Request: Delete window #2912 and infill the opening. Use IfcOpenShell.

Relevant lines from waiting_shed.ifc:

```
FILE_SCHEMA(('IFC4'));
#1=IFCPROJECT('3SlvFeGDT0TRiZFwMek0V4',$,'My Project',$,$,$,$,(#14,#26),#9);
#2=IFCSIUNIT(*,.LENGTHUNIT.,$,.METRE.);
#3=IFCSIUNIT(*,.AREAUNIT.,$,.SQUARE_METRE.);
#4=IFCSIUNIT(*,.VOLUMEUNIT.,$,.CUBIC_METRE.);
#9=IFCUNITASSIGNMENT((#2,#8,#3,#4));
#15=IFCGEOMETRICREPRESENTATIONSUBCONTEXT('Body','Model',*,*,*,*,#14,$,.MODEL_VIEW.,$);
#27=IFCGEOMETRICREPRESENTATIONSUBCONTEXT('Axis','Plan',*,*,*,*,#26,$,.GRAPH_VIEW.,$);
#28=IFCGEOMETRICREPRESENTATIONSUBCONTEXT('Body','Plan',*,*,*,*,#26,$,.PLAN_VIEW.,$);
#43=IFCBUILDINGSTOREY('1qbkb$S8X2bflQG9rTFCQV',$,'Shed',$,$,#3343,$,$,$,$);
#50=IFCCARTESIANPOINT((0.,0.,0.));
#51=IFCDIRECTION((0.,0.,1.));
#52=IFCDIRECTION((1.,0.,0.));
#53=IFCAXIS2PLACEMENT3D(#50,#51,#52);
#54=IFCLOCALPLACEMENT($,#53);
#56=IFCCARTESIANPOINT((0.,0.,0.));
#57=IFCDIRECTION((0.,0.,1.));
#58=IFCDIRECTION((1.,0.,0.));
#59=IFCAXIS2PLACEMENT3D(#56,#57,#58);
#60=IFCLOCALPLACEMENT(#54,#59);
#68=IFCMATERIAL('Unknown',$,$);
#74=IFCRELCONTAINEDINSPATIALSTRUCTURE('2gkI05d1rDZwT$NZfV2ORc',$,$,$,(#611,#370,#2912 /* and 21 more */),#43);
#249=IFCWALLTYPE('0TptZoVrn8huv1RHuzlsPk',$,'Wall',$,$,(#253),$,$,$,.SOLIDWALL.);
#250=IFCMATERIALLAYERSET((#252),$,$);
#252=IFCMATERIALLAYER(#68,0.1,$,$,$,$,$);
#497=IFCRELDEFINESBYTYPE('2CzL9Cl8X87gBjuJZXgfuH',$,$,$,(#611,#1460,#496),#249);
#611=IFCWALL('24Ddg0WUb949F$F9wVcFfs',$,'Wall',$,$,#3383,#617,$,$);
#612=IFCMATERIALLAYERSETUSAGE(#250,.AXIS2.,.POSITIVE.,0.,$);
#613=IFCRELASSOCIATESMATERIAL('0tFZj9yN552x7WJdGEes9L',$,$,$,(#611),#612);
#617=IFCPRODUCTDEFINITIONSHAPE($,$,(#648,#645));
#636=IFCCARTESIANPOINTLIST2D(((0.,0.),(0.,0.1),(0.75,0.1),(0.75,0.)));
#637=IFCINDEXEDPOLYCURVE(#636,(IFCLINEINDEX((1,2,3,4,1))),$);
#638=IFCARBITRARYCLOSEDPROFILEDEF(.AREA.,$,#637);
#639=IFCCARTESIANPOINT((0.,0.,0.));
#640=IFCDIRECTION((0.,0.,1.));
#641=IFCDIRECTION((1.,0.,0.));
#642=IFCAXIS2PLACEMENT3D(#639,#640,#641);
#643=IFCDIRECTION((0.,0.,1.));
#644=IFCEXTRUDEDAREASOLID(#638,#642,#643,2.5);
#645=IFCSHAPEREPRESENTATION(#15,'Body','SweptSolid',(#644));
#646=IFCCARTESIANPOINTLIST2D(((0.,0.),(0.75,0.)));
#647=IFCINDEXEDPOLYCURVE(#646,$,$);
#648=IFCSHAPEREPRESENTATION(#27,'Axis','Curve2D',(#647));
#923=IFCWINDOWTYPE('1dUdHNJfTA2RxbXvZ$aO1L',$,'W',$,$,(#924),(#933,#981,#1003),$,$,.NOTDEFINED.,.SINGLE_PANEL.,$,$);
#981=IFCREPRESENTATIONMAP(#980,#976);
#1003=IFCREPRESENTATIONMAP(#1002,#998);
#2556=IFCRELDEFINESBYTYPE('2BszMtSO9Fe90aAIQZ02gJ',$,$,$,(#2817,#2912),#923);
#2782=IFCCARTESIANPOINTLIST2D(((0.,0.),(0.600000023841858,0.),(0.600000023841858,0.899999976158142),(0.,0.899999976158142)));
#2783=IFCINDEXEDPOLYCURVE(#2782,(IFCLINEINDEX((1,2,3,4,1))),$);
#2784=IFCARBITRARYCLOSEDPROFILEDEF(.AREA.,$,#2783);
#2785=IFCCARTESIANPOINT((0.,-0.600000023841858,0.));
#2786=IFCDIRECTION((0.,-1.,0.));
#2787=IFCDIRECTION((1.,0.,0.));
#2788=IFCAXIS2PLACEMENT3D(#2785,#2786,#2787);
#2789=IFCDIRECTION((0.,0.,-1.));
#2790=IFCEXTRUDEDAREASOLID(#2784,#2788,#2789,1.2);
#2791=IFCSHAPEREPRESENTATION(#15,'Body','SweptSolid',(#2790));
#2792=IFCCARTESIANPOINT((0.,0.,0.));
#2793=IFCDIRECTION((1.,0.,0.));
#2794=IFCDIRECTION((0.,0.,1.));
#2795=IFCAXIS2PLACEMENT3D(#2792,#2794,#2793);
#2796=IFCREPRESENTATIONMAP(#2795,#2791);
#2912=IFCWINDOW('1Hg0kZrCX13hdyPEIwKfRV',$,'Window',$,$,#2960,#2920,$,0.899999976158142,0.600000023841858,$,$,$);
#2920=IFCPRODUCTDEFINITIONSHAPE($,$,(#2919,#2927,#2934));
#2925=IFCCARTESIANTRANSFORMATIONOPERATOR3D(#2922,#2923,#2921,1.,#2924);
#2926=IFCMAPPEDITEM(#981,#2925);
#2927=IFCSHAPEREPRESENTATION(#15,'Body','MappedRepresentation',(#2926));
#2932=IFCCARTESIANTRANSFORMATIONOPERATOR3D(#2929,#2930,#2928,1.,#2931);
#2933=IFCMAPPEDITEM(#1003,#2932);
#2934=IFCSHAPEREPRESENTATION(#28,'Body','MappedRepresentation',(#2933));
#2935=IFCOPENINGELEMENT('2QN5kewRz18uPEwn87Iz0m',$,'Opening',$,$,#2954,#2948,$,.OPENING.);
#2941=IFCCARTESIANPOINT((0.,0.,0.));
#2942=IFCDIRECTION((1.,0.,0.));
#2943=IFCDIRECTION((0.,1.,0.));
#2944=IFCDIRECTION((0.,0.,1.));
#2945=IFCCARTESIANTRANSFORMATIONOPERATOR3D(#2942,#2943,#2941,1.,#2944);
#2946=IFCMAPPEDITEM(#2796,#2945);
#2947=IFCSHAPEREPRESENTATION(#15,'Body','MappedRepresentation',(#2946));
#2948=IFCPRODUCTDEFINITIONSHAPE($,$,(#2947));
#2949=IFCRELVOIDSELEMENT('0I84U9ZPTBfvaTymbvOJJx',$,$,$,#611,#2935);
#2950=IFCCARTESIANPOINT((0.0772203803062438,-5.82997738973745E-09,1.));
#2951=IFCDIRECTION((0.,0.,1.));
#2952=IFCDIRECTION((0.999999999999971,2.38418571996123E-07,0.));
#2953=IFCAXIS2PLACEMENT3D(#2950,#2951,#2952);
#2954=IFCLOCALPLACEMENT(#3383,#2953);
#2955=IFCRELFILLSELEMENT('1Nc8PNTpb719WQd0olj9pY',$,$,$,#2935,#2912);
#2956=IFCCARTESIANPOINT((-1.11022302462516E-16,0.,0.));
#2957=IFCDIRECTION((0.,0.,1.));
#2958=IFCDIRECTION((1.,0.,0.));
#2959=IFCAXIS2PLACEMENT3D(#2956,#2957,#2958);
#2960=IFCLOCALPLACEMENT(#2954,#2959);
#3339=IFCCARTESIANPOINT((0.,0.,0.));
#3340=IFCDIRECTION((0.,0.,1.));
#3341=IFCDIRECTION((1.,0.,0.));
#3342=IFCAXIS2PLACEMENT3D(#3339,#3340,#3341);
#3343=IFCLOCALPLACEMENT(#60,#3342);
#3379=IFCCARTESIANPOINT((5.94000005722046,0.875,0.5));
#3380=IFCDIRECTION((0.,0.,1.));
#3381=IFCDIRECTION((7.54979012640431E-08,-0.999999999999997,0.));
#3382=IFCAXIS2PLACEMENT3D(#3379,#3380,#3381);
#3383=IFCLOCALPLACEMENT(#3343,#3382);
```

```python
import ifcopenshell
import ifcopenshell.api.feature
import ifcopenshell.api.root
import ifcopenshell.geom
import ifcopenshell.util.shape

model = ifcopenshell.open("waiting_shed.ifc")
settings = ifcopenshell.geom.settings()


def volume(element):
    """Net volume in cubic metres, openings subtracted."""
    shape = ifcopenshell.geom.create_shape(settings, element)
    return ifcopenshell.util.shape.get_volume(shape.geometry)


window = model.by_guid("1Hg0kZrCX13hdyPEIwKfRV")
opening = window.FillsVoids[0].RelatingOpeningElement
wall = opening.VoidsElements[0].RelatingBuildingElement
before = volume(wall)

ifcopenshell.api.root.remove_product(model, product=window)
ifcopenshell.api.feature.remove_feature(model, feature=opening)

after = volume(wall)

print(f"wall volume {before:.3f} -> {after:.3f} m3")

model.write("waiting_shed_edited.ifc")
```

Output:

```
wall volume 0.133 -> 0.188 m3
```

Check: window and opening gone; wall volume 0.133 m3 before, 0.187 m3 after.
